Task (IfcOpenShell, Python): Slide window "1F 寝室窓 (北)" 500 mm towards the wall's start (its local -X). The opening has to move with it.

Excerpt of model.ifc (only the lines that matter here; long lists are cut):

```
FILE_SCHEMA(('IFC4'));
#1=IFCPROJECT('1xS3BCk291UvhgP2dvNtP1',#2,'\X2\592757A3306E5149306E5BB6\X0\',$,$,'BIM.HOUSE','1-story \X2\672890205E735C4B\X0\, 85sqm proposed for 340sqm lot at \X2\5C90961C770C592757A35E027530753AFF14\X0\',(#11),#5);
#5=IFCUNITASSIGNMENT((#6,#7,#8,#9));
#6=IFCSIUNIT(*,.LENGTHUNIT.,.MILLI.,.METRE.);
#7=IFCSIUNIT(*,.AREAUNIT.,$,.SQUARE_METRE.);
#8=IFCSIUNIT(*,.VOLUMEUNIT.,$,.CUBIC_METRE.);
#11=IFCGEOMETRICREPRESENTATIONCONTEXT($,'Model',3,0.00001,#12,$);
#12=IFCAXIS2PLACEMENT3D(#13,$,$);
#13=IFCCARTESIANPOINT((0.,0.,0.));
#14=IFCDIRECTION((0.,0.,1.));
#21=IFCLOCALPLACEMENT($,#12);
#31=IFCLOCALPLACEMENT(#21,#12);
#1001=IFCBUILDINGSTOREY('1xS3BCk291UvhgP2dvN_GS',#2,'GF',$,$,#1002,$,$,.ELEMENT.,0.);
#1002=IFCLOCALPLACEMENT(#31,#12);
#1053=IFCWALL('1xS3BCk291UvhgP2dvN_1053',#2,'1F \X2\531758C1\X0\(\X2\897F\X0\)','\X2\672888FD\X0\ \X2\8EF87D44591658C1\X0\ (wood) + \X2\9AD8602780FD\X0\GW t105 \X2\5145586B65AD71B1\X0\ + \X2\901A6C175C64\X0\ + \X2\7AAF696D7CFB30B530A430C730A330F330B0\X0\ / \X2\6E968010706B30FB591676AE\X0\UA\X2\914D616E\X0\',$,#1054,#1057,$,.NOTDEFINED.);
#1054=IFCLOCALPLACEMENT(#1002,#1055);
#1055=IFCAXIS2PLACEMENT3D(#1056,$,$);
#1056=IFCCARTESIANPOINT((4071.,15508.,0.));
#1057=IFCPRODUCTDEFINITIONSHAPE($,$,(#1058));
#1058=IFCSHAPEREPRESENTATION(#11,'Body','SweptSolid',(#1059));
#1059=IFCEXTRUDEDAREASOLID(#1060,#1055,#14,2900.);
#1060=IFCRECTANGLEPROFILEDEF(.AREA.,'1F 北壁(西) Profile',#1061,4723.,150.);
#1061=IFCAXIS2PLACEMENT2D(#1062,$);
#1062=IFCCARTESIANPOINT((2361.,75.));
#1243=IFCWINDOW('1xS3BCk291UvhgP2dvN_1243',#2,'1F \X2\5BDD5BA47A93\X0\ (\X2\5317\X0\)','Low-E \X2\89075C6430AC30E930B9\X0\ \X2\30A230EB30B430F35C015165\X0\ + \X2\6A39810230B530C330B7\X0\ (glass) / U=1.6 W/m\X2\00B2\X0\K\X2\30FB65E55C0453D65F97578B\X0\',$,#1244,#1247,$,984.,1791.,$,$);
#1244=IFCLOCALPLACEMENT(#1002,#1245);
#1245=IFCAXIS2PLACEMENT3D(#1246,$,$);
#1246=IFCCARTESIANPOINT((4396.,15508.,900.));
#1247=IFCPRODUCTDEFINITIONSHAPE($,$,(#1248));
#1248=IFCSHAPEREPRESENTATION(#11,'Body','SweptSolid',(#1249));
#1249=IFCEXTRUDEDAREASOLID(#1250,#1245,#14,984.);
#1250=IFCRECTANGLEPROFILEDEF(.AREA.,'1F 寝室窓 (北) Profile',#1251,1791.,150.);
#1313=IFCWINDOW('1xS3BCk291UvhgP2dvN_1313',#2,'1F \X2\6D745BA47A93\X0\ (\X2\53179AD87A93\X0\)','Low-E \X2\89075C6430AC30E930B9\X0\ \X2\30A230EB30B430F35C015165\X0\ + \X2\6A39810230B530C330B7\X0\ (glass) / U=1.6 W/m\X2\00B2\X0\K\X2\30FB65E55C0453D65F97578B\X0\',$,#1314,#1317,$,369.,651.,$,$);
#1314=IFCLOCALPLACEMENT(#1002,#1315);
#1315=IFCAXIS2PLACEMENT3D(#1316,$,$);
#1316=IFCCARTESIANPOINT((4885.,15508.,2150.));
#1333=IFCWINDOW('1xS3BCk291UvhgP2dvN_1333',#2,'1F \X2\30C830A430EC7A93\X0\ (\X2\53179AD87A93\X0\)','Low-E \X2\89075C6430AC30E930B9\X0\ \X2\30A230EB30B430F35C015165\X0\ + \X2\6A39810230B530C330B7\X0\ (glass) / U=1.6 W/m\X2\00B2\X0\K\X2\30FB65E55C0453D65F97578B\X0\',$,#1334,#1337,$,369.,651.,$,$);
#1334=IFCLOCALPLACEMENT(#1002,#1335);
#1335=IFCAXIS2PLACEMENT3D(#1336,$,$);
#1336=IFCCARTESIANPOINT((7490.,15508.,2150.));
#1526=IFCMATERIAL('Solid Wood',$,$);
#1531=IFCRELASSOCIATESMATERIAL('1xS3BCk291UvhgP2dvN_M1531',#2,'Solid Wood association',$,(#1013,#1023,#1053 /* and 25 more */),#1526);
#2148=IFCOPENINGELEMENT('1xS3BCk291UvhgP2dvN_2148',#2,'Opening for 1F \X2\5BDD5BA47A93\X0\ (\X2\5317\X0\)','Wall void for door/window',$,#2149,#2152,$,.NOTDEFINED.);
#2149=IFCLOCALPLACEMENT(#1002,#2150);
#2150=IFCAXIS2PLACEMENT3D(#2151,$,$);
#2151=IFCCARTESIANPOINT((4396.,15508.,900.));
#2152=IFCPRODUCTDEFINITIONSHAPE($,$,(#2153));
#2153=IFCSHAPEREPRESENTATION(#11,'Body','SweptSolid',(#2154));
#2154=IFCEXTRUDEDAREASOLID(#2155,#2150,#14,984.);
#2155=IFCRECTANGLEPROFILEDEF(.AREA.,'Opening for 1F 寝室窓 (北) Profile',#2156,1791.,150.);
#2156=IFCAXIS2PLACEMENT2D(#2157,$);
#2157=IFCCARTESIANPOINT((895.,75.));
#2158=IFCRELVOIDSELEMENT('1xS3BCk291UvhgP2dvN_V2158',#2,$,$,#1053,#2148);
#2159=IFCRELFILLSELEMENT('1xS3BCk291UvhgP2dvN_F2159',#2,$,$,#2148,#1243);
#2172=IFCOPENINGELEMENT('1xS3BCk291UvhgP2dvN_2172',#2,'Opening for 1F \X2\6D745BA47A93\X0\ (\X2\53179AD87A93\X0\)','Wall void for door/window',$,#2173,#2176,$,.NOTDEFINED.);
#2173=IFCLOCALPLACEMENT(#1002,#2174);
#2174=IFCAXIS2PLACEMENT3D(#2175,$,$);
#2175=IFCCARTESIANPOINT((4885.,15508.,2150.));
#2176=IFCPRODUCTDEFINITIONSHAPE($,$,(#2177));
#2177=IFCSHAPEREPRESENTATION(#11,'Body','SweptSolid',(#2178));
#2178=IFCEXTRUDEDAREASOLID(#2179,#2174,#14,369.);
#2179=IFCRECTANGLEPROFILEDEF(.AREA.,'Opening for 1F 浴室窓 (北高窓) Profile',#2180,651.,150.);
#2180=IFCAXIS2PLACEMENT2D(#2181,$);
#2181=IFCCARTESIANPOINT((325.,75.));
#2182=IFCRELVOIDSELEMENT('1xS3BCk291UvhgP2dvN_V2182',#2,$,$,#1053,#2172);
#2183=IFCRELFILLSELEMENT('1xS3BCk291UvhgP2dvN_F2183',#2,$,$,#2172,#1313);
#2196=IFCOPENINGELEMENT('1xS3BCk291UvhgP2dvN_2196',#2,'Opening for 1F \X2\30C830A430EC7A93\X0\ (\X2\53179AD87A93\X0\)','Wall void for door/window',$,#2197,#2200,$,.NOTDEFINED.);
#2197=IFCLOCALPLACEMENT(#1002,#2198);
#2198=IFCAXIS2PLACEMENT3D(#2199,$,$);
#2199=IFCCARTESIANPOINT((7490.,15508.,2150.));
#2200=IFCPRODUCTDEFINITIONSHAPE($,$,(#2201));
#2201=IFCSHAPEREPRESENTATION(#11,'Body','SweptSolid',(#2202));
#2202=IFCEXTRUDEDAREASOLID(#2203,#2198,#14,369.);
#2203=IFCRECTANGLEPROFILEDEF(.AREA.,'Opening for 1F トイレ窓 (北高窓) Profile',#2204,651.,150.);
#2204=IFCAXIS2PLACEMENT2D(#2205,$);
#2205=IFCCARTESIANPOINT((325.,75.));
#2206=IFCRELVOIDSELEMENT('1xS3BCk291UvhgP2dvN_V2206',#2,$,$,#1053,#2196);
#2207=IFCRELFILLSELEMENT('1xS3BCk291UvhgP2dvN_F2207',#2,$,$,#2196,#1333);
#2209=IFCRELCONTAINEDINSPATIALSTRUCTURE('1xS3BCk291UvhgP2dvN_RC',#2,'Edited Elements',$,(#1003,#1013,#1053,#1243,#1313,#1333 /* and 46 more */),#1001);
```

```python
import ifcopenshell
import ifcopenshell.api.geometry
import ifcopenshell.util.placement
import ifcopenshell.util.unit

model = ifcopenshell.open("model.ifc")
unit_scale = ifcopenshell.util.unit.calculate_unit_scale(model)

window = model.by_id(1243)
opening = window.FillsVoids[0].RelatingOpeningElement
wall = opening.VoidsElements[0].RelatingBuildingElement

wall_matrix = ifcopenshell.util.placement.get_local_placement(wall.ObjectPlacement)
shift = wall_matrix[:3, 0] * -0.5 / unit_scale
before = ifcopenshell.util.placement.get_local_placement(window.ObjectPlacement)[:3, 3].copy()

# The window is not placed relative to its opening, so move both.
for product in (opening, window):
    matrix = ifcopenshell.util.placement.get_local_placement(product.ObjectPlacement)
    matrix[:3, 3] += shift
    ifcopenshell.api.geometry.edit_object_placement(model, product=product, matrix=matrix, is_si=False)

after = ifcopenshell.util.placement.get_local_placement(window.ObjectPlacement)[:3, 3]
print("window moved by", (after - before).round(3) + 0.0)

model.write("model-out.ifc")
```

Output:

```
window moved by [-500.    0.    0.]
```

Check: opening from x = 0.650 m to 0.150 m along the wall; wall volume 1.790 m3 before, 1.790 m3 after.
